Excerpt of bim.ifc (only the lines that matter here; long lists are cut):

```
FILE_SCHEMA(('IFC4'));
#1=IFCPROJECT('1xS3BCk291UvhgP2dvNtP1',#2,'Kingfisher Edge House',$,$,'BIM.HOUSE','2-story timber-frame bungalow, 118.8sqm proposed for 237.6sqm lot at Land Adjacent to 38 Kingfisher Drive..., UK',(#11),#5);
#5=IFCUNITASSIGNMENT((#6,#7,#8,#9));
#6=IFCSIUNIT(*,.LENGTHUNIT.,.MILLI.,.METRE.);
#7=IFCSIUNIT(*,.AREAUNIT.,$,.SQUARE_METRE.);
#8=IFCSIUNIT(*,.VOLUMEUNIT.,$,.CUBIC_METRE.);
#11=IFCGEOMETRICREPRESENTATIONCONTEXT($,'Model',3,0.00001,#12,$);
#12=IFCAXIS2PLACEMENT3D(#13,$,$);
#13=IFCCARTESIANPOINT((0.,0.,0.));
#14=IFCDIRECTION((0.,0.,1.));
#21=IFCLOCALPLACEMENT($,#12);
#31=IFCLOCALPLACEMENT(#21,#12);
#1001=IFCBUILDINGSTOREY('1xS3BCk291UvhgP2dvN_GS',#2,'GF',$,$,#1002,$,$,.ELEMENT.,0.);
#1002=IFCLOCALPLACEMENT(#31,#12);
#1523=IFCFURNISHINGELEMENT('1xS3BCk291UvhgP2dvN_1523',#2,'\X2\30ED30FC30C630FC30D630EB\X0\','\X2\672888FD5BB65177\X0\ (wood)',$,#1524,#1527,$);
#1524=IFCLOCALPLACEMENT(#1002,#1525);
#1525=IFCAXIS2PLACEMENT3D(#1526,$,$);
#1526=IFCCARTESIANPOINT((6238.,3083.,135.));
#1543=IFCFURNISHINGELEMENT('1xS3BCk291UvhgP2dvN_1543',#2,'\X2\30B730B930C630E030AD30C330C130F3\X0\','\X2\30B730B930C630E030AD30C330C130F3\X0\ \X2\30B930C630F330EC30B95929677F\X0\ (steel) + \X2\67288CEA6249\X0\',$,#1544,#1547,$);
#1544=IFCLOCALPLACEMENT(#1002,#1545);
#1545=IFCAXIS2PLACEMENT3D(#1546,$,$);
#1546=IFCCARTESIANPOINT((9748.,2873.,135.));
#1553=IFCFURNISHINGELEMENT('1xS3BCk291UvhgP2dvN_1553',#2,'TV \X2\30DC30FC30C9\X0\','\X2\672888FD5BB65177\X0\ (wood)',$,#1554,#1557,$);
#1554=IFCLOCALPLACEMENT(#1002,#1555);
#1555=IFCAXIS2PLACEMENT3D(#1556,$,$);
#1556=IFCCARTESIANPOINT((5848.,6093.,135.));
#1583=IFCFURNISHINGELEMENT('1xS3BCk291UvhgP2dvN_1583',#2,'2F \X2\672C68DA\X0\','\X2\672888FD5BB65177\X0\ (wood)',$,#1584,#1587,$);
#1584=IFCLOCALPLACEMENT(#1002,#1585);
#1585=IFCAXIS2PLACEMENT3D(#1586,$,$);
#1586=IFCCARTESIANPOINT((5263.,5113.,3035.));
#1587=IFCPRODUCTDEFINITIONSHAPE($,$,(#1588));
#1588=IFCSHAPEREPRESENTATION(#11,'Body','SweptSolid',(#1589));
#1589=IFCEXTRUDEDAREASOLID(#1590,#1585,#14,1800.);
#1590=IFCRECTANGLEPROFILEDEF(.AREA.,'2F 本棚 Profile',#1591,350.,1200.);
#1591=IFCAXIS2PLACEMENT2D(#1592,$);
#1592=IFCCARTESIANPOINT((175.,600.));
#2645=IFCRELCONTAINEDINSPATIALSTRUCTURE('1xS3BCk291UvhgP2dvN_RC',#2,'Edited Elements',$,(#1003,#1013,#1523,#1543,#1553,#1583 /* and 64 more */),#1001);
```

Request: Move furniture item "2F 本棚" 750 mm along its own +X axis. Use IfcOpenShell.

```python
import ifcopenshell
import ifcopenshell.api.geometry
import ifcopenshell.util.placement
import ifcopenshell.util.unit

model = ifcopenshell.open("bim.ifc")
unit_scale = ifcopenshell.util.unit.calculate_unit_scale(model)

item = model.by_id(1583)
matrix = ifcopenshell.util.placement.get_local_placement(item.ObjectPlacement)
matrix[:3, 3] += matrix[:3, 0] * 0.75 / unit_scale
ifcopenshell.api.geometry.edit_object_placement(model, product=item, matrix=matrix, is_si=False)

print(ifcopenshell.util.placement.get_local_placement(item.ObjectPlacement).round(3) + 0.0)

model.write("bim_v2.ifc")
```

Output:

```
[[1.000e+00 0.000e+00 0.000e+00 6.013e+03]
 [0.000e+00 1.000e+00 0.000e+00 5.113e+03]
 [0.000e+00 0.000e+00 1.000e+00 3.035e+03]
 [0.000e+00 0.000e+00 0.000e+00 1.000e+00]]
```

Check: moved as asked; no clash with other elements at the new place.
